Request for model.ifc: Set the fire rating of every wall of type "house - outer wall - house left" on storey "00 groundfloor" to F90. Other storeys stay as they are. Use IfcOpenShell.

First a look at what the model holds.

```python
import ifcopenshell
import ifcopenshell.util.element

model = ifcopenshell.open("model.ifc")
print(model.schema)
storey = next(s for s in model.by_type("IfcBuildingStorey") if s.Name == "00 groundfloor")
walls = [e for e in ifcopenshell.util.element.get_decomposition(storey) if e.is_a("IfcWall")]
seen = {}
for e in walls:
    element_type = ifcopenshell.util.element.get_type(e)
    key = (element_type.Name if element_type != e and element_type else None, ifcopenshell.util.element.get_pset(e, "Pset_WallCommon", "FireRating"))
    seen[key] = seen.get(key, 0) + 1
for (name, value), count in sorted(seen.items(), key=str):
    print(count, "x", name, "|", value)
```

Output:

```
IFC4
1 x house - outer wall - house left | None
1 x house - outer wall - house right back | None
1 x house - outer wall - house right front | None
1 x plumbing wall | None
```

```python
import ifcopenshell
import ifcopenshell.api.pset
import ifcopenshell.util.element

model = ifcopenshell.open("model.ifc")

storey = next(s for s in model.by_type("IfcBuildingStorey") if s.Name == "00 groundfloor")
walls = [e for e in ifcopenshell.util.element.get_decomposition(storey) if e.is_a("IfcWall")]

count = 0
for e in walls:
    element_type = ifcopenshell.util.element.get_type(e)
    if element_type in (None, e) or element_type.Name != "house - outer wall - house left":
        continue
    # add_pset returns the element's existing set when there is one.
    pset = ifcopenshell.api.pset.add_pset(model, product=e, name="Pset_WallCommon")
    ifcopenshell.api.pset.edit_pset(model, pset=pset, properties={"FireRating": "F90"})
    count += 1

print(count, "walls updated")

model.write("model_rev.ifc")
```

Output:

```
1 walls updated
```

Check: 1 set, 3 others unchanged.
